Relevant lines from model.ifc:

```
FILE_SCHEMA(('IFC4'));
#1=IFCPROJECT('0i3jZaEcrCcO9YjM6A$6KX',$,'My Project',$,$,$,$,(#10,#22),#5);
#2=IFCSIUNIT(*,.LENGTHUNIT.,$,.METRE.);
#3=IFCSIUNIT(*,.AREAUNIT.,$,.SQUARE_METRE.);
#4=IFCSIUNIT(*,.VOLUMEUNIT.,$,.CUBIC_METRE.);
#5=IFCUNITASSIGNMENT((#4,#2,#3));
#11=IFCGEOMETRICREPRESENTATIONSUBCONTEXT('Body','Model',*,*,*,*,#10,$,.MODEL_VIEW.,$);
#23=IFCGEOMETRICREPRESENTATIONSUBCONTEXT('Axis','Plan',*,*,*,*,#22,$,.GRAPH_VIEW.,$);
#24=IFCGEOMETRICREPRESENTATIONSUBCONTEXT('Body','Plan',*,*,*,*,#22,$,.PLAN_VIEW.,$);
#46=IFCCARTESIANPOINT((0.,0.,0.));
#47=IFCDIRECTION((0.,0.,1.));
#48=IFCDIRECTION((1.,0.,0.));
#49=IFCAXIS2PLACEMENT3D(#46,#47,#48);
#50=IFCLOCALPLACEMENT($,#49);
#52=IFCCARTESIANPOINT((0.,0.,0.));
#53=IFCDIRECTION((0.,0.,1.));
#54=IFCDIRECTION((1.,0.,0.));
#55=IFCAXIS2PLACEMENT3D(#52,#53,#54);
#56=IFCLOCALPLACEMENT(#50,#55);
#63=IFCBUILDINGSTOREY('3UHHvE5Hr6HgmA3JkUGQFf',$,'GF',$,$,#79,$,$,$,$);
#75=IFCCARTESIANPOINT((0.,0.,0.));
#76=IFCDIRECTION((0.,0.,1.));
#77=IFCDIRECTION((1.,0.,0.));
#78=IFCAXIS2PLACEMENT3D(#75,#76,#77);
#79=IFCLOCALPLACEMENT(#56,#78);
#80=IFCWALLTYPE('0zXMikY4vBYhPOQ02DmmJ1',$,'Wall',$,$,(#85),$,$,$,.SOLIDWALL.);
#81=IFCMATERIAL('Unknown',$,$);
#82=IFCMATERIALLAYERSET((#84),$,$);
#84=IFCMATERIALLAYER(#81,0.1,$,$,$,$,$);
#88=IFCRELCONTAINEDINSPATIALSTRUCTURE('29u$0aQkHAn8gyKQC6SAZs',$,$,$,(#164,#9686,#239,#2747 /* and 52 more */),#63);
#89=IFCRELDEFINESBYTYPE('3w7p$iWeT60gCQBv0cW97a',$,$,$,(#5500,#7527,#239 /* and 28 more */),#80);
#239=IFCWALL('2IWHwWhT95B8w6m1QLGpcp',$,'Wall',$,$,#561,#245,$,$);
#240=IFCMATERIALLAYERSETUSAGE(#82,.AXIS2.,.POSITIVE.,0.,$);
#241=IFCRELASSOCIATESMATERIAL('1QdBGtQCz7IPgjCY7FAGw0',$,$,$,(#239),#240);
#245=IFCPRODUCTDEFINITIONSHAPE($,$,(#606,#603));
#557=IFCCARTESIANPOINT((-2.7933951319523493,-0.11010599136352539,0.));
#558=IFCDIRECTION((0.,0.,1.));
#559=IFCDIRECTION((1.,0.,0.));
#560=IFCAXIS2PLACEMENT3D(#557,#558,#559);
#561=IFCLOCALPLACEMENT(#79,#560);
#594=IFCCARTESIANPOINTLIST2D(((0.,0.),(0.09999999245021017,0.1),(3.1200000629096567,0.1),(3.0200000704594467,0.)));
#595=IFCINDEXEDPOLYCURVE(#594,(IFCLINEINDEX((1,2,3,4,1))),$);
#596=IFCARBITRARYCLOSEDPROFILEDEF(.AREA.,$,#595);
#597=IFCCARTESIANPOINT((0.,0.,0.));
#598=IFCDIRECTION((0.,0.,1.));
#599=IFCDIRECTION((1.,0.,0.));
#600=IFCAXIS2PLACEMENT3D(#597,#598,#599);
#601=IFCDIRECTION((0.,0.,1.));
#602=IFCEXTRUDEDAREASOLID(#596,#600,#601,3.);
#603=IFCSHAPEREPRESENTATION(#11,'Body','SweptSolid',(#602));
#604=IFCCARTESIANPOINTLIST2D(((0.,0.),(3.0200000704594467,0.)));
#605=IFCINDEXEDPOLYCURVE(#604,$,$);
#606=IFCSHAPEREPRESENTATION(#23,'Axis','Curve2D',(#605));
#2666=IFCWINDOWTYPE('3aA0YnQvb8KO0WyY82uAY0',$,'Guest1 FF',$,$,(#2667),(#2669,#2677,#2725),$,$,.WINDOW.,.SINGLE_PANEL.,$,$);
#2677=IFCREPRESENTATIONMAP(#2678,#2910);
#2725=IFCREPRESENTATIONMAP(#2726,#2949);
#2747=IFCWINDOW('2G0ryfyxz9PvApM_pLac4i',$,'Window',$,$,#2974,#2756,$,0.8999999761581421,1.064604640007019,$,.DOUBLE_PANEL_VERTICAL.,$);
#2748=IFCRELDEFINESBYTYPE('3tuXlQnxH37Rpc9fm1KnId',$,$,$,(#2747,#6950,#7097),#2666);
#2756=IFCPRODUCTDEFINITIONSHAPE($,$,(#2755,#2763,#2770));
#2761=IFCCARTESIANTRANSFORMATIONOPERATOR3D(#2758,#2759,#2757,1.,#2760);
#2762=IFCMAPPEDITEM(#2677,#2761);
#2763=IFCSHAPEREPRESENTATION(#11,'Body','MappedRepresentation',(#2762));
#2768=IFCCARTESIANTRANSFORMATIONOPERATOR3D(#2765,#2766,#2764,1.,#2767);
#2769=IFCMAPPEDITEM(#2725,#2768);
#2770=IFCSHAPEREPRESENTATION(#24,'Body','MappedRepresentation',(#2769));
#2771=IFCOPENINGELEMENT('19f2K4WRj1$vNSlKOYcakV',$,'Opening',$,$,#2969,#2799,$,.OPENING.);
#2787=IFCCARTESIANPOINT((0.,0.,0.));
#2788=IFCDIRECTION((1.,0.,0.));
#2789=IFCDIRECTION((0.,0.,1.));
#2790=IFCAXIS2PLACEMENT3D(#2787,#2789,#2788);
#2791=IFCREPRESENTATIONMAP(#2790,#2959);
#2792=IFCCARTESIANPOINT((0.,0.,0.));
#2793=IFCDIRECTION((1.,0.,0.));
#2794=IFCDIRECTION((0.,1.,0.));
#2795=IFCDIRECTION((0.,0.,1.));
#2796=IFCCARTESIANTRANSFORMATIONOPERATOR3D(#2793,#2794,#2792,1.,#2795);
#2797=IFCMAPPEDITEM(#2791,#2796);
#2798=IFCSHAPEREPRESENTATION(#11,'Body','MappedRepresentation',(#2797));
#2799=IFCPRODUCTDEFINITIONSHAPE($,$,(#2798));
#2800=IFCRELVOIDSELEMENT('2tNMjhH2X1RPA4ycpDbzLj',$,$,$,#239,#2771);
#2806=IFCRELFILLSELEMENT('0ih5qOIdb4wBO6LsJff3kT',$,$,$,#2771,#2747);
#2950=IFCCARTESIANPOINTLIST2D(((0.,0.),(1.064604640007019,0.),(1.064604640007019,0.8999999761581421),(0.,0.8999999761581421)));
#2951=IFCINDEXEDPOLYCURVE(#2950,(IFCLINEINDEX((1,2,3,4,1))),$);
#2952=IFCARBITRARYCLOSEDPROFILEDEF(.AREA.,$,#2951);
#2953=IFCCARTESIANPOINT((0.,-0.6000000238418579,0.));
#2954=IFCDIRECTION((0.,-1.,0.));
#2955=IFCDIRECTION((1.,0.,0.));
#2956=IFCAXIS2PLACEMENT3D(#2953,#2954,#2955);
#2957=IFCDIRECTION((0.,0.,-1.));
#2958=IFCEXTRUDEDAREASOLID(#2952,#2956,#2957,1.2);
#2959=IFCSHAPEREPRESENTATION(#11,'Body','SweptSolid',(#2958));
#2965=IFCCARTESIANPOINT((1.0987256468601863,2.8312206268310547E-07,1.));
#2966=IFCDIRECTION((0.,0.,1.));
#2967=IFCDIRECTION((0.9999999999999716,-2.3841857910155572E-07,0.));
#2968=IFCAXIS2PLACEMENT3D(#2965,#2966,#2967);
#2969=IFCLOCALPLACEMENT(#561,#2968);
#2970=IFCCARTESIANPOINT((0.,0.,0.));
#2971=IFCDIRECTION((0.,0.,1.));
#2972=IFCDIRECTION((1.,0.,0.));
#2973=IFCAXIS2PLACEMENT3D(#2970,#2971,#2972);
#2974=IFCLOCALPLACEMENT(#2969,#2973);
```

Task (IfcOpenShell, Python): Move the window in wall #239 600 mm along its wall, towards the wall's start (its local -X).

```python
import ifcopenshell
import ifcopenshell.api.geometry
import ifcopenshell.util.placement
import ifcopenshell.util.unit

model = ifcopenshell.open("model.ifc")
unit_scale = ifcopenshell.util.unit.calculate_unit_scale(model)

window = model.by_guid("2G0ryfyxz9PvApM_pLac4i")
opening = window.FillsVoids[0].RelatingOpeningElement
wall = opening.VoidsElements[0].RelatingBuildingElement

wall_matrix = ifcopenshell.util.placement.get_local_placement(wall.ObjectPlacement)
shift = wall_matrix[:3, 0] * -0.6 / unit_scale
before = ifcopenshell.util.placement.get_local_placement(window.ObjectPlacement)[:3, 3].copy()

# The window is placed relative to its opening, so it follows when the opening moves.
matrix = ifcopenshell.util.placement.get_local_placement(opening.ObjectPlacement)
matrix[:3, 3] += shift
ifcopenshell.api.geometry.edit_object_placement(
    model, product=opening, matrix=matrix, is_si=False, should_transform_children=True
)

after = ifcopenshell.util.placement.get_local_placement(window.ObjectPlacement)[:3, 3]
print("window moved by", (after - before).round(3) + 0.0)

model.write("model_v2.ifc")
```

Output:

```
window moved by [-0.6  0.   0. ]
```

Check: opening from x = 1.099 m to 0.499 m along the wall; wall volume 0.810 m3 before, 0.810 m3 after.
